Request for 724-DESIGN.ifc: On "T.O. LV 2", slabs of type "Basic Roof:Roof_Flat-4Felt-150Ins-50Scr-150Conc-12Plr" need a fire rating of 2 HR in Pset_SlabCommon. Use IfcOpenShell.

First a look at what the model holds.

```python
import ifcopenshell
import ifcopenshell.util.element

model = ifcopenshell.open("724-DESIGN.ifc")
print(model.schema)
storey = next(s for s in model.by_type("IfcBuildingStorey") if s.Name == "T.O. LV 2")
slabs = [e for e in ifcopenshell.util.element.get_decomposition(storey) if e.is_a("IfcSlab")]
seen = {}
for e in slabs:
    element_type = ifcopenshell.util.element.get_type(e)
    key = (element_type.Name if element_type != e and element_type else None, ifcopenshell.util.element.get_pset(e, "Pset_SlabCommon", "FireRating"))
    seen[key] = seen.get(key, 0) + 1
for (name, value), count in sorted(seen.items(), key=str):
    print(count, "x", name, "|", value)
```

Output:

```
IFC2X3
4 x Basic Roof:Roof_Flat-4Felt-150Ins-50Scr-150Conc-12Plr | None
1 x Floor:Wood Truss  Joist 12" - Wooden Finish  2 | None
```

```python
import ifcopenshell
import ifcopenshell.api.pset
import ifcopenshell.util.element

model = ifcopenshell.open("724-DESIGN.ifc")

storey = next(s for s in model.by_type("IfcBuildingStorey") if s.Name == "T.O. LV 2")
slabs = [e for e in ifcopenshell.util.element.get_decomposition(storey) if e.is_a("IfcSlab")]

count = 0
for e in slabs:
    element_type = ifcopenshell.util.element.get_type(e)
    if element_type in (None, e) or element_type.Name != "Basic Roof:Roof_Flat-4Felt-150Ins-50Scr-150Conc-12Plr":
        continue
    # add_pset returns the element's existing set when there is one.
    pset = ifcopenshell.api.pset.add_pset(model, product=e, name="Pset_SlabCommon")
    ifcopenshell.api.pset.edit_pset(model, pset=pset, properties={"FireRating": "2 HR"})
    count += 1

print(count, "slabs updated")

model.write("724-DESIGN_edited.ifc")
```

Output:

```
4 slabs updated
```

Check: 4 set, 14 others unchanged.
